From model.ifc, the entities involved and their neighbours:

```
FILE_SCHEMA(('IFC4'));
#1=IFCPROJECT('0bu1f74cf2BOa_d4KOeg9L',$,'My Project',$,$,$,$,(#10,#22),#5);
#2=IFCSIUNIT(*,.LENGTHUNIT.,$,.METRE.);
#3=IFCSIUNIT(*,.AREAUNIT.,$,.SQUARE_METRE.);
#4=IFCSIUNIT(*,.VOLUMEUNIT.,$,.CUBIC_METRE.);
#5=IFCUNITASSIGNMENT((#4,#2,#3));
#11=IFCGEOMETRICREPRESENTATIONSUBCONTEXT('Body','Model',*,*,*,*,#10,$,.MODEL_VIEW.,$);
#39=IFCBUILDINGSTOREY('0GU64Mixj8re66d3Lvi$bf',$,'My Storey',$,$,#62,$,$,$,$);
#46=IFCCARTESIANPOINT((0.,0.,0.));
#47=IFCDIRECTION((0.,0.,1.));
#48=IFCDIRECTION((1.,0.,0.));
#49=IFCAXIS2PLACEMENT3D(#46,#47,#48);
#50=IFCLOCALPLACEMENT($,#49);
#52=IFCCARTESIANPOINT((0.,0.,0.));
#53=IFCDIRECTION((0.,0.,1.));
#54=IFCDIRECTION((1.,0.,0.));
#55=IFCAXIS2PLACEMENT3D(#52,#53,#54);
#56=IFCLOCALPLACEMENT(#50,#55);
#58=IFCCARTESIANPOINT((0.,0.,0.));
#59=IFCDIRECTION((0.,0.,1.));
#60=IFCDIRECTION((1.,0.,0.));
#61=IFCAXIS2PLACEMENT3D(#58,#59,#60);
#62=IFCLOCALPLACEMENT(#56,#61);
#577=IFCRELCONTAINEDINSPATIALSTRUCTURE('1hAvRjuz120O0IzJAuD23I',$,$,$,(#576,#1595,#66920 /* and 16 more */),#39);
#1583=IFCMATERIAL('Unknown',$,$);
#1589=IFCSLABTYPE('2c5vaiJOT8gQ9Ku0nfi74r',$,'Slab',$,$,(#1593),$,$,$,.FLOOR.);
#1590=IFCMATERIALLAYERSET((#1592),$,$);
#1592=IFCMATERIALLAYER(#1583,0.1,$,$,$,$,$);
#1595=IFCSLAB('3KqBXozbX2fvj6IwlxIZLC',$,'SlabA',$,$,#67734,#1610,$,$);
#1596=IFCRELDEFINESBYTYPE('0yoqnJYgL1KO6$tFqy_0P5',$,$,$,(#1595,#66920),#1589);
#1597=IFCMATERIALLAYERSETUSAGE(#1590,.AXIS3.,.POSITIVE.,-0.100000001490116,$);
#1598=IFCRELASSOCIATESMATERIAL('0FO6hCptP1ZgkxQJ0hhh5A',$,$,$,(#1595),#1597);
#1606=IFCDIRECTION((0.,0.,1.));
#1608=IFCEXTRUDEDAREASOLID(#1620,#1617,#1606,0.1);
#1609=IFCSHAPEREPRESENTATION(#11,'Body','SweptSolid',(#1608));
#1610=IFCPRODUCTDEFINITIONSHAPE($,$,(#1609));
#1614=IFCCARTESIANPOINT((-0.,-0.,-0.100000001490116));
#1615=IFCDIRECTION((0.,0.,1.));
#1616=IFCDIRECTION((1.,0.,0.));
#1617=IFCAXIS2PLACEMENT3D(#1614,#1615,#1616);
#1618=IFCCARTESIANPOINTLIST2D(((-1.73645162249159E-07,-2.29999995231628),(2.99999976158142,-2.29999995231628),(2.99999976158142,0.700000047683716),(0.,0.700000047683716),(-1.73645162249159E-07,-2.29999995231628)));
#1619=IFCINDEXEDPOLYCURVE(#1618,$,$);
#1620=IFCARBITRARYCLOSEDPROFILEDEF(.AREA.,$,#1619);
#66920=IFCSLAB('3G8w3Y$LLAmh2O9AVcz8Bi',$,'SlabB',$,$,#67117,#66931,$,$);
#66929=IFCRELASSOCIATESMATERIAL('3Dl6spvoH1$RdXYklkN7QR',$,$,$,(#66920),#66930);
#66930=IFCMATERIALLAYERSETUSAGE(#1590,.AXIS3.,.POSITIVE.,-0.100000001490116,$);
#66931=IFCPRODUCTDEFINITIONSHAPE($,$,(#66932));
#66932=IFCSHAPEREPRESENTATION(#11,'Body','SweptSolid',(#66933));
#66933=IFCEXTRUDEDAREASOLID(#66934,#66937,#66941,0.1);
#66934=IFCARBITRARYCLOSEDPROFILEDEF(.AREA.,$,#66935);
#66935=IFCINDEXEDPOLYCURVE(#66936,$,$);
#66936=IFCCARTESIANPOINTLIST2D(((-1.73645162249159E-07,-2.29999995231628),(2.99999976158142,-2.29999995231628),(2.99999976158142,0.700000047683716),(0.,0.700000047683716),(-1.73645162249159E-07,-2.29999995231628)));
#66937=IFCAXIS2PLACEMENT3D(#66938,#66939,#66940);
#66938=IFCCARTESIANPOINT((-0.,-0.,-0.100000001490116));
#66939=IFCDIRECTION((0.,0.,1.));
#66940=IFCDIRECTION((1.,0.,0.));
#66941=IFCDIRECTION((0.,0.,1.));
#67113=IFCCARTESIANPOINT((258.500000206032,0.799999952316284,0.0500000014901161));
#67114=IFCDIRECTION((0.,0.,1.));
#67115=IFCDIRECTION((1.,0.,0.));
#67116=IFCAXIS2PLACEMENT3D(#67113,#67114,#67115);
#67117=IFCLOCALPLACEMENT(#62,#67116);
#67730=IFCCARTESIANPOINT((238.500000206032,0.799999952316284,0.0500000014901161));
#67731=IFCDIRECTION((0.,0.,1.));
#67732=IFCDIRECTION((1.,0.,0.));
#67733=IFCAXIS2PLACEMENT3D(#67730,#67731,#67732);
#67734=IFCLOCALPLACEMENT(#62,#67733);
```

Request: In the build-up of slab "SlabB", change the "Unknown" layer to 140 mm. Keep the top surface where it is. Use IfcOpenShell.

```python
import ifcopenshell
import ifcopenshell.util.element
import ifcopenshell.util.representation
import ifcopenshell.util.unit

model = ifcopenshell.open("model.ifc")
unit_scale = ifcopenshell.util.unit.calculate_unit_scale(model)

layer_set = model.by_id(1590)
layer = next(l for l in layer_set.MaterialLayers if l.Material and l.Material.Name == "Unknown")
change = 0.14 / unit_scale - layer.LayerThickness
layer.LayerThickness += change

# The layer set is shared, so every slab that uses it gets the new thickness.
slabs = [e for e in ifcopenshell.util.element.get_elements_by_material(model, layer_set) if e.is_a("IfcSlab")]
for slab in sorted(slabs, key=lambda e: e.id()):
    body = ifcopenshell.util.representation.get_representation(slab, "Model", "Body")
    solid = body.Items[0]
    old_depth = solid.Depth
    solid.Depth += change
    # Extruded upwards: lower the start of the extrusion so the top stays.
    x, y, z = solid.Position.Location.Coordinates
    solid.Position.Location = model.createIfcCartesianPoint((x, y, z - change))
    print(slab.id(), f"{old_depth:g} -> {solid.Depth:g}")

# The layers are counted up from the underside, which has moved.
for usage in {ifcopenshell.util.element.get_material(slab) for slab in slabs}:
    usage.OffsetFromReferenceLine -= change

model.write("model_v2.ifc")
```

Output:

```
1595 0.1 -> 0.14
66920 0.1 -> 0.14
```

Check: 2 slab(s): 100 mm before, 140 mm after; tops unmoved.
